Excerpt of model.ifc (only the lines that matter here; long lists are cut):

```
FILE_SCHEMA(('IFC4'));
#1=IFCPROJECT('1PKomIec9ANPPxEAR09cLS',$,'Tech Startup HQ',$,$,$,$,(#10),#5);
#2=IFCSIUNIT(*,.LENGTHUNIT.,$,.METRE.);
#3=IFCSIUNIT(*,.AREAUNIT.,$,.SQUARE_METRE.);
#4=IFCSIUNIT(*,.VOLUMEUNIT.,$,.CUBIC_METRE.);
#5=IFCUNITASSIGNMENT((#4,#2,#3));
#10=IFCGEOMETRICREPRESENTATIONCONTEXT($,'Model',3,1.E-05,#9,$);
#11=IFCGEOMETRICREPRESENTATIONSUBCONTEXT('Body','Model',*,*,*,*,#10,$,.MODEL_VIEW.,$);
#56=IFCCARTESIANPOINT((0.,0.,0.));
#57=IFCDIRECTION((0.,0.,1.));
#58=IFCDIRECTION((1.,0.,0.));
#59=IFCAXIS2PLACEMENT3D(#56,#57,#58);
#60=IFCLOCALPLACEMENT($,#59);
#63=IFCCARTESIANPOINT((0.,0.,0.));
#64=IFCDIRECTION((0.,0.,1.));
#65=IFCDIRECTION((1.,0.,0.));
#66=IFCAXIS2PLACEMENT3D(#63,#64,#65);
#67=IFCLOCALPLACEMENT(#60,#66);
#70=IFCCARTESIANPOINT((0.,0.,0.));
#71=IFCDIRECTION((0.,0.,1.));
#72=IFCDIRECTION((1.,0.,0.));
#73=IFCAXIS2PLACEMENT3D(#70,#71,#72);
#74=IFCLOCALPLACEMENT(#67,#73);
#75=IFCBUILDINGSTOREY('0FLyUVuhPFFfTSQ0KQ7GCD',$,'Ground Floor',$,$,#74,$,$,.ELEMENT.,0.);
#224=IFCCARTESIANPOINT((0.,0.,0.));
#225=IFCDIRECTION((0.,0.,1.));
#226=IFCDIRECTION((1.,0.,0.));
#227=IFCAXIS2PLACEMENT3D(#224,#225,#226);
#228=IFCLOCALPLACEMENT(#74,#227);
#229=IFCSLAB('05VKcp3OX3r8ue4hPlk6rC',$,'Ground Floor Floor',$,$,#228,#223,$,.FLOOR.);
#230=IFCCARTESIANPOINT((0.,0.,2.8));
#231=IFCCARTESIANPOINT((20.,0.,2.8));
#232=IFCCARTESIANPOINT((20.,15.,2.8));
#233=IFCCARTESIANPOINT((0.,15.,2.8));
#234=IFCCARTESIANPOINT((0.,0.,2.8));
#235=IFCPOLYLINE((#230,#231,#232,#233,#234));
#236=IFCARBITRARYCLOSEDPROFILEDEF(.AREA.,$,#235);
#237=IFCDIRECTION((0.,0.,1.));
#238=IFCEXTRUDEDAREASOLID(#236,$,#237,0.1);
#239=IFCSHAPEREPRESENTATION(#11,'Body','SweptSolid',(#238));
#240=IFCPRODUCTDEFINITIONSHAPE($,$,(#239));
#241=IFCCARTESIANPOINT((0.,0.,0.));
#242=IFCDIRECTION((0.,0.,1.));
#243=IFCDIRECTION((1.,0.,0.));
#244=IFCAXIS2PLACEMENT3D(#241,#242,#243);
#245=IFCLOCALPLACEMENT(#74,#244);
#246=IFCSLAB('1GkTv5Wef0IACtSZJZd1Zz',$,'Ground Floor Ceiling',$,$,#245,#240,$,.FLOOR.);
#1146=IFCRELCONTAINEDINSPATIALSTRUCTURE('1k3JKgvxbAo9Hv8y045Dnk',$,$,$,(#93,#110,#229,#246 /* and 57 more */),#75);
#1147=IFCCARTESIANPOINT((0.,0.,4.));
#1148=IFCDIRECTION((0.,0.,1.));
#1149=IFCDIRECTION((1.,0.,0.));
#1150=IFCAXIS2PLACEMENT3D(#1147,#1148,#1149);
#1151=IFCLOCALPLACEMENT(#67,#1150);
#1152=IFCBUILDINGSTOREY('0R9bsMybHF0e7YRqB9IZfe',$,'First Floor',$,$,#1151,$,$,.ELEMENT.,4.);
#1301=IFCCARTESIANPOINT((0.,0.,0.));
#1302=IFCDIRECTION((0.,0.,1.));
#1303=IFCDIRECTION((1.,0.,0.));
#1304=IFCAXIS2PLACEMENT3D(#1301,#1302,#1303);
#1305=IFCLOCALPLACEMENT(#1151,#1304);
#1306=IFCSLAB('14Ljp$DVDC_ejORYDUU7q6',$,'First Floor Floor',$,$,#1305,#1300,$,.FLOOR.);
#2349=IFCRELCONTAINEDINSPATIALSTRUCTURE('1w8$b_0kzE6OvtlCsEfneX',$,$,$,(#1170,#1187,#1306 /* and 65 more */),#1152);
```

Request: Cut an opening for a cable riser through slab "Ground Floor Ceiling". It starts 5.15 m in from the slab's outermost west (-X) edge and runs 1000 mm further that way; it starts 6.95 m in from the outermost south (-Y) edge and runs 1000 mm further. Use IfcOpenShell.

```python
import numpy as np
import ifcopenshell
import ifcopenshell.api.feature
import ifcopenshell.api.geometry
import ifcopenshell.api.root
import ifcopenshell.geom
import ifcopenshell.util.placement
import ifcopenshell.util.representation
import ifcopenshell.util.shape
import ifcopenshell.util.unit

model = ifcopenshell.open("model.ifc")
unit_scale = ifcopenshell.util.unit.calculate_unit_scale(model)
settings = ifcopenshell.geom.settings()


def volume(element):
    """Net volume in cubic metres, openings subtracted."""
    shape = ifcopenshell.geom.create_shape(settings, element)
    return ifcopenshell.util.shape.get_volume(shape.geometry)


slab = model.by_guid("1GkTv5Wef0IACtSZJZd1Zz")
before = volume(slab)

# Extent in the slab's own axes, in metres. The edges named are its -X and -Y sides.
slab_shape = ifcopenshell.geom.create_shape(settings, slab)
vertices = ifcopenshell.util.shape.get_vertices(slab_shape.geometry)
x_min, y_min, bottom = vertices.min(axis=0)
top = vertices[:, 2].max()

opening = ifcopenshell.api.root.create_entity(model, ifc_class="IfcOpeningElement", name="Cable riser opening", predefined_type="OPENING")
context = ifcopenshell.util.representation.get_context(model, "Model", "Body", "MODEL_VIEW")
width, depth = 1, 1
outline = [(0.0, 0.0), (width, 0.0), (width, depth), (0.0, depth), (0.0, 0.0)]
# Overshoot both faces by 50 mm so the cut is clean.
shape = ifcopenshell.api.geometry.add_slab_representation(
    model, context=context, depth=top - bottom + 0.1, polyline=outline
)
ifcopenshell.api.geometry.assign_representation(model, product=opening, representation=shape)

matrix = ifcopenshell.util.placement.get_local_placement(slab.ObjectPlacement)
matrix[:, 3] = matrix @ np.append(np.array([x_min + 5.15, y_min + 6.95, bottom - 0.05]) / unit_scale, 1.0)
ifcopenshell.api.geometry.edit_object_placement(model, product=opening, matrix=matrix, is_si=False)
ifcopenshell.api.feature.add_feature(model, feature=opening, element=slab)

after = volume(slab)

print(f"slab volume {before:.3f} -> {after:.3f} m3")

model.write("model_updated.ifc")
```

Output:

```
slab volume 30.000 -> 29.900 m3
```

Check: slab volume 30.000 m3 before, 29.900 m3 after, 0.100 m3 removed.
